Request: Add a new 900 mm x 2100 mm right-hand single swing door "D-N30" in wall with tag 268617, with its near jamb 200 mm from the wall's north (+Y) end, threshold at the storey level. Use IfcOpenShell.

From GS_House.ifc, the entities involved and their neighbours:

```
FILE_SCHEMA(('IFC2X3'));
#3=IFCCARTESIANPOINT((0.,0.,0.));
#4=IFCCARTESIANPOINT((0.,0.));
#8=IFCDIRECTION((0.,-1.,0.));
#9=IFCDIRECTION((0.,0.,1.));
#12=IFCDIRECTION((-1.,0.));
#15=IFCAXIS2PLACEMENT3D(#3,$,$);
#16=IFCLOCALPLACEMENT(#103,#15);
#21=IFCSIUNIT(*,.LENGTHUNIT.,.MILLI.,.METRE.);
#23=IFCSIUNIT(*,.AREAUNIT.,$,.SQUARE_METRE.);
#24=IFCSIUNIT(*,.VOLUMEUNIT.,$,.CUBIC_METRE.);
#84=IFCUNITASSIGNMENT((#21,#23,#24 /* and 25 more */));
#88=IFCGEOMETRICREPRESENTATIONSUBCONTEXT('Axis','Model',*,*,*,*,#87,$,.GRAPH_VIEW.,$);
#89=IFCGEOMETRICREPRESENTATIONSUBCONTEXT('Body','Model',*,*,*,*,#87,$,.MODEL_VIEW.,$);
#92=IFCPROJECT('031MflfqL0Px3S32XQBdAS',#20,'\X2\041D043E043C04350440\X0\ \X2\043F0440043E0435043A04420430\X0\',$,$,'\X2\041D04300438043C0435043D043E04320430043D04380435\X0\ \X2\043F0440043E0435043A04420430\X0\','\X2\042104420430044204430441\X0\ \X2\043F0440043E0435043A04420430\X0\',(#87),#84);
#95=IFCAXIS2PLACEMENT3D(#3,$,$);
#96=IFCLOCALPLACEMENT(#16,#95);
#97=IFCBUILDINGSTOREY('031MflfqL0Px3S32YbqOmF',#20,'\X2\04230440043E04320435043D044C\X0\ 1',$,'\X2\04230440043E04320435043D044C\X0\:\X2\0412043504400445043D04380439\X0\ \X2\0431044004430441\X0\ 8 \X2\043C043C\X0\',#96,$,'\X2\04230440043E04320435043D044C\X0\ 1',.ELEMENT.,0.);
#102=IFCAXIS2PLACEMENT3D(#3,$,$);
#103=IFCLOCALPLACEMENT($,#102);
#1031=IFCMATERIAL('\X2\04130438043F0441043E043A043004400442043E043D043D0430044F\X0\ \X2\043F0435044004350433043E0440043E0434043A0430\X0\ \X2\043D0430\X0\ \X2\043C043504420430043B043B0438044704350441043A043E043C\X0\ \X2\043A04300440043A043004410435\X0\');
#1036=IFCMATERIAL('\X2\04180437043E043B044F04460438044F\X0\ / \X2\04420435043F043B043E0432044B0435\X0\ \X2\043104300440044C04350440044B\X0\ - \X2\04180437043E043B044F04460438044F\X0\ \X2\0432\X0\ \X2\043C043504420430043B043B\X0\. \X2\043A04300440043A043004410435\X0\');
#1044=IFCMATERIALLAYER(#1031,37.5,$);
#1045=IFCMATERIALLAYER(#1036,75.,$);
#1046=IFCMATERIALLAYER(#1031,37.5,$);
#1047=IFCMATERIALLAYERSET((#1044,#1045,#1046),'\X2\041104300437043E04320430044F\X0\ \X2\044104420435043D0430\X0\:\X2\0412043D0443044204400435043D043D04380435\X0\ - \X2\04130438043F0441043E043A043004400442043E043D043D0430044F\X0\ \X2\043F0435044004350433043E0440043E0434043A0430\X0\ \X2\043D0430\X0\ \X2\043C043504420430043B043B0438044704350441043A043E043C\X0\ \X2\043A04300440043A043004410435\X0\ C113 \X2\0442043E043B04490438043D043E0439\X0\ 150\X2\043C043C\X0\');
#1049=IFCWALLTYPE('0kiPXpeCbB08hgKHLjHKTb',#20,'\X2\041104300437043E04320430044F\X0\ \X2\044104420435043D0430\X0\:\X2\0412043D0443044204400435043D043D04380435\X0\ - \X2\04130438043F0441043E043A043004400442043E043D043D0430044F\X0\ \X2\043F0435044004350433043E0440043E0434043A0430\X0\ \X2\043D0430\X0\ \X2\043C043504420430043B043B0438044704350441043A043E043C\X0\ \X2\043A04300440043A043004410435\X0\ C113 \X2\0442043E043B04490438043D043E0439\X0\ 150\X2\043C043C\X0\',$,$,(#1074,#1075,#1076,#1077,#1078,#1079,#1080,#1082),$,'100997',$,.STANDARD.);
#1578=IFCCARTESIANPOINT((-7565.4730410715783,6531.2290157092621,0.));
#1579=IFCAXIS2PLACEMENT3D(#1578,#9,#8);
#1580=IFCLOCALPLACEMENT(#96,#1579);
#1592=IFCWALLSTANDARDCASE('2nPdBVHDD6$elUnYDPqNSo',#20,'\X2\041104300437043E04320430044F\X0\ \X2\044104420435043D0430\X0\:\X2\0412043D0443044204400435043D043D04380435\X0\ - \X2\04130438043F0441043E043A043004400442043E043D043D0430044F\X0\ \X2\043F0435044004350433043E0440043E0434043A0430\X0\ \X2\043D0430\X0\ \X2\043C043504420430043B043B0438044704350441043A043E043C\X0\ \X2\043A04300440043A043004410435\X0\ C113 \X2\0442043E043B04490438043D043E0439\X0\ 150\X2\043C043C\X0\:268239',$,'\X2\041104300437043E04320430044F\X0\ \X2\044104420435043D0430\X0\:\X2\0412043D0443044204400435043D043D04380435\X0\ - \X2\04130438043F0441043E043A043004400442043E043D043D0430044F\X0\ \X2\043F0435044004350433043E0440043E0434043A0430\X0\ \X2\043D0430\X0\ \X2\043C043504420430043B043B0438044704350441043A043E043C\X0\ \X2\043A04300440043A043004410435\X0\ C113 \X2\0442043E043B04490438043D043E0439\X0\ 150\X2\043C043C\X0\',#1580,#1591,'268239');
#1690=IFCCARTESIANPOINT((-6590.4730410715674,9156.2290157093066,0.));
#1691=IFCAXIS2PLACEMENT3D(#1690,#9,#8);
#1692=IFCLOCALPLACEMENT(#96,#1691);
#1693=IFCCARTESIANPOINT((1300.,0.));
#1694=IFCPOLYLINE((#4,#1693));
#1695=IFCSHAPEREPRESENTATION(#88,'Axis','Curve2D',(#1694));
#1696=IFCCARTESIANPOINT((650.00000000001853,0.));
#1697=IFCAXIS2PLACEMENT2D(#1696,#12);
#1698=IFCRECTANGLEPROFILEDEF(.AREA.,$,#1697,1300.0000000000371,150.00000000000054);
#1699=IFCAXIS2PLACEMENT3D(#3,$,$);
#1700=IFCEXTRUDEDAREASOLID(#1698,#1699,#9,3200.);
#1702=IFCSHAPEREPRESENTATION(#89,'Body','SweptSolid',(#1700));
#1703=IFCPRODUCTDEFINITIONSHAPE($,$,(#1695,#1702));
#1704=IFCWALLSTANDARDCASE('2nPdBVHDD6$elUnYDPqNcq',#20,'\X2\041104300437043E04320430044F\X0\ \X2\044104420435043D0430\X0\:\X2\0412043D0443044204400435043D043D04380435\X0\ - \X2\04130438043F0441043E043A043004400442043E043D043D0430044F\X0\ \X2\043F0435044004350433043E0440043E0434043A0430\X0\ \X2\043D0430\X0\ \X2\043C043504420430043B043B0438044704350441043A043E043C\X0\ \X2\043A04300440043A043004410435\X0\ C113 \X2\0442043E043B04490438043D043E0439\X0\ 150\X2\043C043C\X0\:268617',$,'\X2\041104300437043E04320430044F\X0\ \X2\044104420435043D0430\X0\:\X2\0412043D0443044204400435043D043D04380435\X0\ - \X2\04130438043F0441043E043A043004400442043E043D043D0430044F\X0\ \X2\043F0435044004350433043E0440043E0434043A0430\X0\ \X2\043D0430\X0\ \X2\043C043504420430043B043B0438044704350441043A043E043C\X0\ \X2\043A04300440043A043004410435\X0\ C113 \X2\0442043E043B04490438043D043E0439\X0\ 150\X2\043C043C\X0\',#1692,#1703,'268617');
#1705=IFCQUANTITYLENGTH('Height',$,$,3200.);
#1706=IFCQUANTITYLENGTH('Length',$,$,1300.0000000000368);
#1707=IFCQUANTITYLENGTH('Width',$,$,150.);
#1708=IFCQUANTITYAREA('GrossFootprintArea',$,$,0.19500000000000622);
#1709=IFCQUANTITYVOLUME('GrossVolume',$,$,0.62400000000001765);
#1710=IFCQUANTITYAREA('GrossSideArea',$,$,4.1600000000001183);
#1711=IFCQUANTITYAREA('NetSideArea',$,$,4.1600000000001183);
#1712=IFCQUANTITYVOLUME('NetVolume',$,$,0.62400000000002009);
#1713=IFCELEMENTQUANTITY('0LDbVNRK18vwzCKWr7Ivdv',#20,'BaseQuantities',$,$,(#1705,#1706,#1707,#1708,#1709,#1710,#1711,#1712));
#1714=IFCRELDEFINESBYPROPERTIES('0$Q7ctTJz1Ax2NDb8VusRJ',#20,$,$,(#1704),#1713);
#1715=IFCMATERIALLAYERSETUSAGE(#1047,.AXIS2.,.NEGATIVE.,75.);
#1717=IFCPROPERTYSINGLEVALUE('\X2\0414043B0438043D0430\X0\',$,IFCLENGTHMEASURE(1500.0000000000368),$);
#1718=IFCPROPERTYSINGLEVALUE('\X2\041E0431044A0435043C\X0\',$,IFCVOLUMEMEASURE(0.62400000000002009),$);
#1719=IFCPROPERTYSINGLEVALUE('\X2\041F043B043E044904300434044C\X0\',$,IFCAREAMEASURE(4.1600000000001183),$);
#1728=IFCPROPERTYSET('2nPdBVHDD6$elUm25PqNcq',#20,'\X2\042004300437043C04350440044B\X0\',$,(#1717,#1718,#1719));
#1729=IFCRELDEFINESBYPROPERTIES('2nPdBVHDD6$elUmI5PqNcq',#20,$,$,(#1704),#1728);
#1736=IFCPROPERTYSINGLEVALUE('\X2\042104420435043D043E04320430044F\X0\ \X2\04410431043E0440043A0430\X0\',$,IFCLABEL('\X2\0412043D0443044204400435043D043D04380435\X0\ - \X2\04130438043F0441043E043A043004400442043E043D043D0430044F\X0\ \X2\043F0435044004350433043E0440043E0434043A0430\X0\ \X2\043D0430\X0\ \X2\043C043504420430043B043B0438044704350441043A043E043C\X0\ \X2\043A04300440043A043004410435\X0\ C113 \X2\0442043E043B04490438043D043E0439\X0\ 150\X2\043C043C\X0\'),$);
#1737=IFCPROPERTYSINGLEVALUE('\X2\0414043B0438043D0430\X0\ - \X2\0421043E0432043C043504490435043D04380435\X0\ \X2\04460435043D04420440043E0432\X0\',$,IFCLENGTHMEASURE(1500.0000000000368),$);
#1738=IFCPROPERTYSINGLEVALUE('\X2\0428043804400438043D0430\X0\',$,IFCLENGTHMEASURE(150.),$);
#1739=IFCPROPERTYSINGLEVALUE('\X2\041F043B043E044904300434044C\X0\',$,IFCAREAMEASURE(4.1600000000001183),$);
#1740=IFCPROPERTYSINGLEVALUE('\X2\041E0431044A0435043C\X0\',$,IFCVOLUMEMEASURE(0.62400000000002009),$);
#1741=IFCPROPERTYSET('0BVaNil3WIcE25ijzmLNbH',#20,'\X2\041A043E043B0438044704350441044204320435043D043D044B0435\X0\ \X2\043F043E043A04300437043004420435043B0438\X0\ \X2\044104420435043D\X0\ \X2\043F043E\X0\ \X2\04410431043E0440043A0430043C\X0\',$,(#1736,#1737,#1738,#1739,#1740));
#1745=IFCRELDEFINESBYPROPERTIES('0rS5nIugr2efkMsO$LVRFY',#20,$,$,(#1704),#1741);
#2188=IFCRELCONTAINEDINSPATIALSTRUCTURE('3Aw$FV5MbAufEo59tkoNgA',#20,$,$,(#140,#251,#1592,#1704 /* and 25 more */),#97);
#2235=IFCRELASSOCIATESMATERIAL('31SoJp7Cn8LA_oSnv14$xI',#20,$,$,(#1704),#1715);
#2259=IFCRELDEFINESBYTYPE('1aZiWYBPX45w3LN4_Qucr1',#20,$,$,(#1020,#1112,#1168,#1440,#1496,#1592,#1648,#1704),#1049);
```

```python
import numpy as np
import ifcopenshell
import ifcopenshell.api.feature
import ifcopenshell.api.geometry
import ifcopenshell.api.pset
import ifcopenshell.api.root
import ifcopenshell.api.spatial
import ifcopenshell.api.type
import ifcopenshell.geom
import ifcopenshell.util.element
import ifcopenshell.util.placement
import ifcopenshell.util.representation
import ifcopenshell.util.shape
import ifcopenshell.util.unit

model = ifcopenshell.open("GS_House.ifc")
unit_scale = ifcopenshell.util.unit.calculate_unit_scale(model)
area_scale = ifcopenshell.util.unit.calculate_unit_scale(model, "AREAUNIT")
volume_scale = ifcopenshell.util.unit.calculate_unit_scale(model, "VOLUMEUNIT")
settings = ifcopenshell.geom.settings()


def volume(element):
    """Net volume in cubic metres, openings subtracted."""
    shape = ifcopenshell.geom.create_shape(settings, element)
    return ifcopenshell.util.shape.get_volume(shape.geometry)


wall = model.by_id(1704)
storey = ifcopenshell.util.element.get_container(wall, ifc_class="IfcBuildingStorey")
context = ifcopenshell.util.representation.get_context(model, "Model", "Body", "MODEL_VIEW")
before = volume(wall)

width, height, from_end, sill = 0.9, 2.1, 0.2, 0.0  # metres

# The wall runs along its own X axis, and the end named is its -X end.
wall_shape = ifcopenshell.geom.create_shape(settings, wall)
x, y, z = ifcopenshell.util.shape.get_vertices(wall_shape.geometry).T
start = x.min() + from_end
face, thickness = float(y.min()), float(y.max() - y.min())
wall_matrix = ifcopenshell.util.placement.get_local_placement(wall.ObjectPlacement)
level = ifcopenshell.util.placement.get_local_placement(storey.ObjectPlacement)[2, 3]


def in_wall(x, y):
    """Placement at x, y metres in the wall's axes, at sill height."""
    matrix = wall_matrix.copy()
    matrix[:, 3] = wall_matrix @ np.array([x / unit_scale, y / unit_scale, 0.0, 1.0])
    matrix[2, 3] = level + sill / unit_scale
    return matrix


# Opening: a box that overshoots both wall faces by 50 mm.
opening = ifcopenshell.api.root.create_entity(model, ifc_class="IfcOpeningElement")
box = ifcopenshell.api.geometry.add_wall_representation(
    model, context=context, length=width, height=height, thickness=thickness + 0.1
)
ifcopenshell.api.geometry.assign_representation(model, product=opening, representation=box)
ifcopenshell.api.geometry.edit_object_placement(model, product=opening, matrix=in_wall(start, face - 0.05), is_si=False)
ifcopenshell.api.feature.add_feature(model, feature=opening, element=wall)

door = ifcopenshell.api.root.create_entity(model, ifc_class="IfcDoor", name="D-N30")
door.OverallWidth, door.OverallHeight = width / unit_scale, height / unit_scale
body = ifcopenshell.api.geometry.add_door_representation(
    model,
    context=context,
    overall_width=door.OverallWidth,
    overall_height=door.OverallHeight,
    operation_type="SINGLE_SWING_RIGHT",
    lining_properties={"LiningDepth": thickness / unit_scale, "ThresholdDepth": thickness / unit_scale},
)
ifcopenshell.api.geometry.assign_representation(model, product=door, representation=body)
ifcopenshell.api.spatial.assign_container(model, products=[door], relating_structure=storey)
fills = ifcopenshell.api.feature.add_filling(model, opening=opening, element=door)
fills.OwnerHistory = door.OwnerHistory  # required in IFC2X3

# IFC2X3 keeps the operation on the door style.
style = ifcopenshell.api.root.create_entity(model, ifc_class="IfcDoorStyle", name="D-N30")
style.OperationType, style.ConstructionType = "SINGLE_SWING_RIGHT", "NOTDEFINED"
style.ParameterTakesPrecedence = style.Sizeable = False
ifcopenshell.api.type.assign_type(model, related_objects=[door], relating_type=style)

# The lining spans the wall, so the door starts at the wall face.
ifcopenshell.api.geometry.edit_object_placement(model, product=door, matrix=in_wall(start, face), is_si=False)

after = volume(wall)

# Update the wall's stored quantities.
qto = model.by_id(ifcopenshell.util.element.get_pset(wall, "BaseQuantities", should_inherit=False)["id"])
ifcopenshell.api.pset.edit_qto(model, qto=qto, properties={
    "NetSideArea": after / thickness / area_scale,
    "NetVolume": after / volume_scale,
})
pset = model.by_id(ifcopenshell.util.element.get_pset(wall, "Размеры", should_inherit=False)["id"])
ifcopenshell.api.pset.edit_pset(model, pset=pset, properties={
    "Объем": model.create_entity("IfcVolumeMeasure", after / volume_scale),
    "Площадь": model.create_entity("IfcAreaMeasure", after / thickness / area_scale),
})
pset = model.by_id(ifcopenshell.util.element.get_pset(wall, "Количественные показатели стен по сборкам", should_inherit=False)["id"])
ifcopenshell.api.pset.edit_pset(model, pset=pset, properties={
    "Площадь": model.create_entity("IfcAreaMeasure", after / thickness / area_scale),
    "Объем": model.create_entity("IfcVolumeMeasure", after / volume_scale),
})

print(f"wall volume {before:.3f} -> {after:.3f} m3")

model.write("GS_House_rev.ifc")
```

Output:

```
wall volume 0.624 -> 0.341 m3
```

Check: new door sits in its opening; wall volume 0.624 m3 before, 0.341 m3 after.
